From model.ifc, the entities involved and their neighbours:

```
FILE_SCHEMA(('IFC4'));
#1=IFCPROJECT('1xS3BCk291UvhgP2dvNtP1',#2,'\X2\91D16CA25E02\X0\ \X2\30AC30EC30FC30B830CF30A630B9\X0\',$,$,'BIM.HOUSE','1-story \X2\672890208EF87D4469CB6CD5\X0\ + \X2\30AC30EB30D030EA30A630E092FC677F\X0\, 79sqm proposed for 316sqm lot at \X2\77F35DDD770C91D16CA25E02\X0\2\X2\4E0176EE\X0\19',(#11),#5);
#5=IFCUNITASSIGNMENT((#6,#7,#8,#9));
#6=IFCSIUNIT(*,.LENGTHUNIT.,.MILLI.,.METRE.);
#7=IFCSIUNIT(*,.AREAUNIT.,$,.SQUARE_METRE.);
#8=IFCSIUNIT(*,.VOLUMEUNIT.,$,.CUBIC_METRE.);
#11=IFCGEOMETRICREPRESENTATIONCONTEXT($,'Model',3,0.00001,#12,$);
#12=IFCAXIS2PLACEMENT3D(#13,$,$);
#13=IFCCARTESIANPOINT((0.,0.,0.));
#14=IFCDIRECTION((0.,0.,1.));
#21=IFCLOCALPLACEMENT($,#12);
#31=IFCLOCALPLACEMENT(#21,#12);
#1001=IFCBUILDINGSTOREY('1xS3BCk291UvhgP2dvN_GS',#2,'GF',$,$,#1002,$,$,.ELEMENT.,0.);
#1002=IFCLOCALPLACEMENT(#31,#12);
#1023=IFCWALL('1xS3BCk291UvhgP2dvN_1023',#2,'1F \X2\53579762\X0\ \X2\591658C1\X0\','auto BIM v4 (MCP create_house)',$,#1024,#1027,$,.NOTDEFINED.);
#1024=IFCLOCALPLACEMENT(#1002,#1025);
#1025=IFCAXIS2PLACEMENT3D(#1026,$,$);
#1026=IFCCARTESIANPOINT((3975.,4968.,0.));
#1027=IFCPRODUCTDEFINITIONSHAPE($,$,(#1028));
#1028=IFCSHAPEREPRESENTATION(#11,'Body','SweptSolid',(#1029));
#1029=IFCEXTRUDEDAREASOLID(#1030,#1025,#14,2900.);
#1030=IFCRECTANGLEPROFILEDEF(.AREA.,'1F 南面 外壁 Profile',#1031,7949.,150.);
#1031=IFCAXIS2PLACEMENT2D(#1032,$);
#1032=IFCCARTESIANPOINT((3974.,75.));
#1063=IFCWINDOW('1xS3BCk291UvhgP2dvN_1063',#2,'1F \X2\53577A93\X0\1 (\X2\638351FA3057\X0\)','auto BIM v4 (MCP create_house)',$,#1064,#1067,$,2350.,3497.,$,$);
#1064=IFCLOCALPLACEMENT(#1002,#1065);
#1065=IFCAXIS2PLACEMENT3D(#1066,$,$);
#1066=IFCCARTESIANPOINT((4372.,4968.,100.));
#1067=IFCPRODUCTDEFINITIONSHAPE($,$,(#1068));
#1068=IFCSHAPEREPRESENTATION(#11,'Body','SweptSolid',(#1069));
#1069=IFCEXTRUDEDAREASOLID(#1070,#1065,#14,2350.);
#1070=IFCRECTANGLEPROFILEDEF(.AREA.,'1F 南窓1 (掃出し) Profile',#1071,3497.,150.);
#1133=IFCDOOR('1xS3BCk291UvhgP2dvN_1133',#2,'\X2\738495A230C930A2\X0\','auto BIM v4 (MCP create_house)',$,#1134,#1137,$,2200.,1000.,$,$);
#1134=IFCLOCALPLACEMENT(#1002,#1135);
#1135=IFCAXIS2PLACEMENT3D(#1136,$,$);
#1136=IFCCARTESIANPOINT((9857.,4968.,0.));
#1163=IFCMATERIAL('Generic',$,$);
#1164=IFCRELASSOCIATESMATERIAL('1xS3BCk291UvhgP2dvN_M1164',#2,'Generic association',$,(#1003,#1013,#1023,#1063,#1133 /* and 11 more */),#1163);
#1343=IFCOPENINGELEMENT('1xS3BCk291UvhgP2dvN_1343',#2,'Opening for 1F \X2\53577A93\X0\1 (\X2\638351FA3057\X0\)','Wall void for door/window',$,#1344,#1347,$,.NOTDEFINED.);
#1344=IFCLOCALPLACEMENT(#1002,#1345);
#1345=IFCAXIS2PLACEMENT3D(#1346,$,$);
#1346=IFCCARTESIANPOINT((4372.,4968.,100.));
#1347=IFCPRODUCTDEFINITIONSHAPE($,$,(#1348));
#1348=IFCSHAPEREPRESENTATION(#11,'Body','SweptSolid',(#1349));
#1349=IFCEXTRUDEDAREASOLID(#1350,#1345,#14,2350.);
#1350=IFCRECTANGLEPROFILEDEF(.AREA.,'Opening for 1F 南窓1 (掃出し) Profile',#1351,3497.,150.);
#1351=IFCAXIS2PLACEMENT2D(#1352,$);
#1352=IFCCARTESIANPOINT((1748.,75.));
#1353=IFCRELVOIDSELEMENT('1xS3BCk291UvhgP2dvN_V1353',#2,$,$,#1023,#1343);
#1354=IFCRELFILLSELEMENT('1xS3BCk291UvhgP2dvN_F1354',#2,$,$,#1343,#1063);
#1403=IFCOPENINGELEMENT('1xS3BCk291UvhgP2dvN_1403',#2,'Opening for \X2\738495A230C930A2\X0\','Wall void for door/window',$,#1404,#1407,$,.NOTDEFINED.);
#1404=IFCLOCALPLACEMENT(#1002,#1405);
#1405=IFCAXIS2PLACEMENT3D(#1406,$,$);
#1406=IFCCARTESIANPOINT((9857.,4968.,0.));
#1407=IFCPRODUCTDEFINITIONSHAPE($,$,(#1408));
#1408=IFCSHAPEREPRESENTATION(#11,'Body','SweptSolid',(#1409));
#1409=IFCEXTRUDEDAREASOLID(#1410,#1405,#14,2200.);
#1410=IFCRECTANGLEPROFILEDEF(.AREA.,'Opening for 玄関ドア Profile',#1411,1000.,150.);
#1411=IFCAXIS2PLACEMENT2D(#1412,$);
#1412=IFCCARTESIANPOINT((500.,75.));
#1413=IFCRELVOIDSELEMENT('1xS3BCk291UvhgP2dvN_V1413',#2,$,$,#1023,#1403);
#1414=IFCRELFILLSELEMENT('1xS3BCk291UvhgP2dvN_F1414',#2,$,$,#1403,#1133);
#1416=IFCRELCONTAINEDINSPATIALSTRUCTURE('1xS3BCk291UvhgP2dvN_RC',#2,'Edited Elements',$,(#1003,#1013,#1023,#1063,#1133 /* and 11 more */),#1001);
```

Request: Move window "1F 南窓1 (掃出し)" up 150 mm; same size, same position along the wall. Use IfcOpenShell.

```python
import numpy as np
import ifcopenshell
import ifcopenshell.api.geometry
import ifcopenshell.util.placement
import ifcopenshell.util.unit

model = ifcopenshell.open("model.ifc")
unit_scale = ifcopenshell.util.unit.calculate_unit_scale(model)

window = model.by_guid("1xS3BCk291UvhgP2dvN_1063")
opening = window.FillsVoids[0].RelatingOpeningElement
dz = 0.15 / unit_scale

shift = np.array([0.0, 0.0, dz])
# The window is not placed relative to its opening, so move both.
for product in (opening, window):
    matrix = ifcopenshell.util.placement.get_local_placement(product.ObjectPlacement)
    matrix[:3, 3] += shift
    ifcopenshell.api.geometry.edit_object_placement(model, product=product, matrix=matrix, is_si=False)

print(f"moved by {dz * unit_scale:+.3f} m")

model.write("model-out.ifc")
```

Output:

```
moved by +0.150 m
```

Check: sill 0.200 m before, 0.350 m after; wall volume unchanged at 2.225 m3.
